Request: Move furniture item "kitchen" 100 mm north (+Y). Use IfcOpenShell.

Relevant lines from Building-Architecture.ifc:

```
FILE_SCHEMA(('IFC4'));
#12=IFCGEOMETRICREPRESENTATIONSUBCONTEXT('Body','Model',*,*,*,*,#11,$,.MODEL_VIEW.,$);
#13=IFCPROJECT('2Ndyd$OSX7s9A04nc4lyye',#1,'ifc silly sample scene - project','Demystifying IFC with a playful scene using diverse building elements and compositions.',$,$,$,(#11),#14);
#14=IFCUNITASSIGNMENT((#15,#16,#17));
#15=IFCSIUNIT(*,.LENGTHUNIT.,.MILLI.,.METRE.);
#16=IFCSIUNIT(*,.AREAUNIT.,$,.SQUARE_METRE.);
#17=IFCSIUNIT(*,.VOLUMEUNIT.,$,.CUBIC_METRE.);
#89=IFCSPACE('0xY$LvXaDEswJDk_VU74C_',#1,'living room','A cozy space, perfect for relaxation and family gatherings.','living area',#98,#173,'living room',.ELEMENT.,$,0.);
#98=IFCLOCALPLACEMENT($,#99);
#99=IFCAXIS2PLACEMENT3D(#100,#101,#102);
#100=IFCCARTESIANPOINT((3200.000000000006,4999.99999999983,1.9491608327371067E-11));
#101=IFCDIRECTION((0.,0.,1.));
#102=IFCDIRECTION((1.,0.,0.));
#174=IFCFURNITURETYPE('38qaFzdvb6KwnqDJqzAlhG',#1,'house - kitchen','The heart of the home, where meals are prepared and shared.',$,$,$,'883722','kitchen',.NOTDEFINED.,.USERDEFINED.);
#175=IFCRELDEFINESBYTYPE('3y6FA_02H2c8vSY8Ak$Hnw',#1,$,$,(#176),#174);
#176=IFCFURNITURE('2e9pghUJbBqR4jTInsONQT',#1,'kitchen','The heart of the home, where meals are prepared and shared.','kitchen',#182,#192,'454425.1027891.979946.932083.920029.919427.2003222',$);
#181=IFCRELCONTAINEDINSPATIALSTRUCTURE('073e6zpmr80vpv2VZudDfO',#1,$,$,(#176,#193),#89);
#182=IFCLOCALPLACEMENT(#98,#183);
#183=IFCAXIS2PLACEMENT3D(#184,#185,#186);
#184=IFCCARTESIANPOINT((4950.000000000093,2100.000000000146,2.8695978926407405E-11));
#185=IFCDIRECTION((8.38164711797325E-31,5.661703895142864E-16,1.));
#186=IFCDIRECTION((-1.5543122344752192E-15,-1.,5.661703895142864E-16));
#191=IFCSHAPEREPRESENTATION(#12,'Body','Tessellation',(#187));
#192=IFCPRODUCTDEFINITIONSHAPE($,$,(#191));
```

```python
import ifcopenshell
import ifcopenshell.api.geometry
import ifcopenshell.util.placement

model = ifcopenshell.open("Building-Architecture.ifc")

item = model.by_guid("2e9pghUJbBqR4jTInsONQT")
matrix = ifcopenshell.util.placement.get_local_placement(item.ObjectPlacement)
matrix[1, 3] += 100.0
ifcopenshell.api.geometry.edit_object_placement(model, product=item, matrix=matrix, is_si=False)

print(ifcopenshell.util.placement.get_local_placement(item.ObjectPlacement).round(3) + 0.0)

model.write("Building-Architecture_edited.ifc")
```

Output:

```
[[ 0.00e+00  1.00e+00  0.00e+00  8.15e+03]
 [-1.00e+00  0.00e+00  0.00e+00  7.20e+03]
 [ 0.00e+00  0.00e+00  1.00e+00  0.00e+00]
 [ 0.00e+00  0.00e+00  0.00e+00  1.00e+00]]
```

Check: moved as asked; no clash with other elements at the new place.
